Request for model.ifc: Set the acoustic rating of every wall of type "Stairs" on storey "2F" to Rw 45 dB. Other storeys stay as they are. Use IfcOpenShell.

First a look at what the model holds.

```python
import ifcopenshell
import ifcopenshell.util.element

model = ifcopenshell.open("model.ifc")
print(model.schema)
storey = next(s for s in model.by_type("IfcBuildingStorey") if s.Name == "2F")
walls = [e for e in ifcopenshell.util.element.get_decomposition(storey) if e.is_a("IfcWall")]
seen = {}
for e in walls:
    element_type = ifcopenshell.util.element.get_type(e)
    key = (element_type.Name if element_type != e and element_type else None, ifcopenshell.util.element.get_pset(e, "Pset_WallCommon", "AcousticRating"))
    seen[key] = seen.get(key, 0) + 1
for (name, value), count in sorted(seen.items(), key=str):
    print(count, "x", name, "|", value)
```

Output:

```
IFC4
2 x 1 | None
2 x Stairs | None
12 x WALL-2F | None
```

```python
import ifcopenshell
import ifcopenshell.api.pset
import ifcopenshell.util.element

model = ifcopenshell.open("model.ifc")

storey = next(s for s in model.by_type("IfcBuildingStorey") if s.Name == "2F")
walls = [e for e in ifcopenshell.util.element.get_decomposition(storey) if e.is_a("IfcWall")]

count = 0
for e in walls:
    element_type = ifcopenshell.util.element.get_type(e)
    if element_type in (None, e) or element_type.Name != "Stairs":
        continue
    # add_pset returns the element's existing set when there is one.
    pset = ifcopenshell.api.pset.add_pset(model, product=e, name="Pset_WallCommon")
    ifcopenshell.api.pset.edit_pset(model, pset=pset, properties={"AcousticRating": "Rw 45 dB"})
    count += 1

print(count, "walls updated")

model.write("model_rev.ifc")
```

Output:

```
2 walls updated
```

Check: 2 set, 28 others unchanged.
